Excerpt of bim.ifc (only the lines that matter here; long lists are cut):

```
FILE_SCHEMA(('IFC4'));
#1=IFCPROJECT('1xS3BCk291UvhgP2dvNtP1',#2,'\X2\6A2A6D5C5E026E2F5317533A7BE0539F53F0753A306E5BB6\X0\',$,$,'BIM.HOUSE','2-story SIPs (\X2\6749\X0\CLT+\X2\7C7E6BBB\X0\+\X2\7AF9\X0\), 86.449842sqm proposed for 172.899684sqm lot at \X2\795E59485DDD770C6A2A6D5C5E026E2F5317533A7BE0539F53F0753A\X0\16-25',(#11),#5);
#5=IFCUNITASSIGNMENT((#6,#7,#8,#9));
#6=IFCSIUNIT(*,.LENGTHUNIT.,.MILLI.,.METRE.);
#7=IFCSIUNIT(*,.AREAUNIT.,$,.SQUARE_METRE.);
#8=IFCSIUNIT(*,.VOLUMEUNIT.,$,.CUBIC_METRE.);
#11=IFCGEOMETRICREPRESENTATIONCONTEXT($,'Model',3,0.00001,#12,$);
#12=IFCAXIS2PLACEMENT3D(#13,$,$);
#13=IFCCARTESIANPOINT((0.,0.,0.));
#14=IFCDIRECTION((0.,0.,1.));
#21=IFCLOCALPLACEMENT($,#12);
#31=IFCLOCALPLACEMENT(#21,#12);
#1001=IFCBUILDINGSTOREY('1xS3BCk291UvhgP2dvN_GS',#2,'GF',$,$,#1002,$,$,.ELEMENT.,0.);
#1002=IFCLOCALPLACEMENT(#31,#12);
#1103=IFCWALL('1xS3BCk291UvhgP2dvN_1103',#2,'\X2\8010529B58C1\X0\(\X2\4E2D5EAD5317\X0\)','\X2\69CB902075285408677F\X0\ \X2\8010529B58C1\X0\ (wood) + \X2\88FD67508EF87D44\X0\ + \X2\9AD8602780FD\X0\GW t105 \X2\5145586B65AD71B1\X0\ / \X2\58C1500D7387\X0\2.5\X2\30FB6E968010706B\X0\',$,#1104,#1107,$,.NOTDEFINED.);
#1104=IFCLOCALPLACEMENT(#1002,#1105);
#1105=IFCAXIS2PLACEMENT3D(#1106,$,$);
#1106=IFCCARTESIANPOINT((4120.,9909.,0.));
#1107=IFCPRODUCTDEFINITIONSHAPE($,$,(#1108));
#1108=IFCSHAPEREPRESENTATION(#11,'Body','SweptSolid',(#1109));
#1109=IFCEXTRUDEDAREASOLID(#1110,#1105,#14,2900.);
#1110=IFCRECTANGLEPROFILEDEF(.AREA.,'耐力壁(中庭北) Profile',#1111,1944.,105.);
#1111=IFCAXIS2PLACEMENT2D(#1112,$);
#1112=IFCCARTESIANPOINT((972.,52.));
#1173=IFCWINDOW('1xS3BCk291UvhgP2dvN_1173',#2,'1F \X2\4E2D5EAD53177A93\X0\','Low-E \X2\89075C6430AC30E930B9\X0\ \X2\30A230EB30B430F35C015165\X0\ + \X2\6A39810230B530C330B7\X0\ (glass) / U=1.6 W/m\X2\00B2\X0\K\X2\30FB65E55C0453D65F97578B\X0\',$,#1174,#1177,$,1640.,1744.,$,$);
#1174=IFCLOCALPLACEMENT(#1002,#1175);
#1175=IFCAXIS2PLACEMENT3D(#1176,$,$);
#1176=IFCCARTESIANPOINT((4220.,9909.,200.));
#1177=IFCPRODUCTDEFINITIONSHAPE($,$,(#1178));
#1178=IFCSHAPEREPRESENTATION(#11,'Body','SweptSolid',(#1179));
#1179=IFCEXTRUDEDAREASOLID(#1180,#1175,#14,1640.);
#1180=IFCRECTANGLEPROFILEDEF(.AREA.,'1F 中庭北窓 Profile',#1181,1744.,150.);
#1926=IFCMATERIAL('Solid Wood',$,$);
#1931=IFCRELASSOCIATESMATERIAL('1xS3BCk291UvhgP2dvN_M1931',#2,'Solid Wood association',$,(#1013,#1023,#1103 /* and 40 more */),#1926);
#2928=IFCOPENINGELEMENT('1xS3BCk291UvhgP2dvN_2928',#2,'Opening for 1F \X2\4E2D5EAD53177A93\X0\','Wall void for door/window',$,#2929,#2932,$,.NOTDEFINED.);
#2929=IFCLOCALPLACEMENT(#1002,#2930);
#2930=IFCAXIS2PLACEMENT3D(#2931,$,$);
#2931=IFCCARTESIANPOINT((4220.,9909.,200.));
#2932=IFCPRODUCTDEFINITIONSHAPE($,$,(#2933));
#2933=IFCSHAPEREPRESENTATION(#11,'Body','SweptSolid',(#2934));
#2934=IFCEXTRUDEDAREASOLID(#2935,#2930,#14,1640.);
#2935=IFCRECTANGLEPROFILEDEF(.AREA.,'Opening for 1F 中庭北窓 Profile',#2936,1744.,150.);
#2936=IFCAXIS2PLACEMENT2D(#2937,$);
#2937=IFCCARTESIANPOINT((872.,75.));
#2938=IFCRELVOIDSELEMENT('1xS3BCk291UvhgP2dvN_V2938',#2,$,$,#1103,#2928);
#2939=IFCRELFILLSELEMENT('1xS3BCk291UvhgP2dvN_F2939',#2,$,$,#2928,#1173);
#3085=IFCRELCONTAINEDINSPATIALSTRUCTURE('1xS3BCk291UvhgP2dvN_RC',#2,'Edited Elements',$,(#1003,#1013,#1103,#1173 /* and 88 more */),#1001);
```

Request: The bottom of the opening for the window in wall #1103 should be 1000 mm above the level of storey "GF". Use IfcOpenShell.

```python
import numpy as np
import ifcopenshell
import ifcopenshell.api.geometry
import ifcopenshell.geom
import ifcopenshell.util.element
import ifcopenshell.util.placement
import ifcopenshell.util.shape
import ifcopenshell.util.unit

model = ifcopenshell.open("bim.ifc")
unit_scale = ifcopenshell.util.unit.calculate_unit_scale(model)

window = model.by_guid("1xS3BCk291UvhgP2dvN_1173")
opening = window.FillsVoids[0].RelatingOpeningElement
storey = ifcopenshell.util.element.get_container(window, ifc_class="IfcBuildingStorey")
level = ifcopenshell.util.placement.get_local_placement(storey.ObjectPlacement)[2, 3]

# The opening's origin need not be at the sill, so measure its lowest point.
shape = ifcopenshell.geom.create_shape(ifcopenshell.geom.settings(), opening)
bottom = ifcopenshell.util.shape.get_shape_bottom_elevation(shape, shape.geometry) / unit_scale
dz = level + 1000.0 - bottom

shift = np.array([0.0, 0.0, dz])
# The window is not placed relative to its opening, so move both.
for product in (opening, window):
    matrix = ifcopenshell.util.placement.get_local_placement(product.ObjectPlacement)
    matrix[:3, 3] += shift
    ifcopenshell.api.geometry.edit_object_placement(model, product=product, matrix=matrix, is_si=False)

print(f"moved by {dz * unit_scale:+.3f} m")

model.write("bim_updated.ifc")
```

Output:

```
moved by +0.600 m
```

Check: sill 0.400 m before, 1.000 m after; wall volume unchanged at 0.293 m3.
